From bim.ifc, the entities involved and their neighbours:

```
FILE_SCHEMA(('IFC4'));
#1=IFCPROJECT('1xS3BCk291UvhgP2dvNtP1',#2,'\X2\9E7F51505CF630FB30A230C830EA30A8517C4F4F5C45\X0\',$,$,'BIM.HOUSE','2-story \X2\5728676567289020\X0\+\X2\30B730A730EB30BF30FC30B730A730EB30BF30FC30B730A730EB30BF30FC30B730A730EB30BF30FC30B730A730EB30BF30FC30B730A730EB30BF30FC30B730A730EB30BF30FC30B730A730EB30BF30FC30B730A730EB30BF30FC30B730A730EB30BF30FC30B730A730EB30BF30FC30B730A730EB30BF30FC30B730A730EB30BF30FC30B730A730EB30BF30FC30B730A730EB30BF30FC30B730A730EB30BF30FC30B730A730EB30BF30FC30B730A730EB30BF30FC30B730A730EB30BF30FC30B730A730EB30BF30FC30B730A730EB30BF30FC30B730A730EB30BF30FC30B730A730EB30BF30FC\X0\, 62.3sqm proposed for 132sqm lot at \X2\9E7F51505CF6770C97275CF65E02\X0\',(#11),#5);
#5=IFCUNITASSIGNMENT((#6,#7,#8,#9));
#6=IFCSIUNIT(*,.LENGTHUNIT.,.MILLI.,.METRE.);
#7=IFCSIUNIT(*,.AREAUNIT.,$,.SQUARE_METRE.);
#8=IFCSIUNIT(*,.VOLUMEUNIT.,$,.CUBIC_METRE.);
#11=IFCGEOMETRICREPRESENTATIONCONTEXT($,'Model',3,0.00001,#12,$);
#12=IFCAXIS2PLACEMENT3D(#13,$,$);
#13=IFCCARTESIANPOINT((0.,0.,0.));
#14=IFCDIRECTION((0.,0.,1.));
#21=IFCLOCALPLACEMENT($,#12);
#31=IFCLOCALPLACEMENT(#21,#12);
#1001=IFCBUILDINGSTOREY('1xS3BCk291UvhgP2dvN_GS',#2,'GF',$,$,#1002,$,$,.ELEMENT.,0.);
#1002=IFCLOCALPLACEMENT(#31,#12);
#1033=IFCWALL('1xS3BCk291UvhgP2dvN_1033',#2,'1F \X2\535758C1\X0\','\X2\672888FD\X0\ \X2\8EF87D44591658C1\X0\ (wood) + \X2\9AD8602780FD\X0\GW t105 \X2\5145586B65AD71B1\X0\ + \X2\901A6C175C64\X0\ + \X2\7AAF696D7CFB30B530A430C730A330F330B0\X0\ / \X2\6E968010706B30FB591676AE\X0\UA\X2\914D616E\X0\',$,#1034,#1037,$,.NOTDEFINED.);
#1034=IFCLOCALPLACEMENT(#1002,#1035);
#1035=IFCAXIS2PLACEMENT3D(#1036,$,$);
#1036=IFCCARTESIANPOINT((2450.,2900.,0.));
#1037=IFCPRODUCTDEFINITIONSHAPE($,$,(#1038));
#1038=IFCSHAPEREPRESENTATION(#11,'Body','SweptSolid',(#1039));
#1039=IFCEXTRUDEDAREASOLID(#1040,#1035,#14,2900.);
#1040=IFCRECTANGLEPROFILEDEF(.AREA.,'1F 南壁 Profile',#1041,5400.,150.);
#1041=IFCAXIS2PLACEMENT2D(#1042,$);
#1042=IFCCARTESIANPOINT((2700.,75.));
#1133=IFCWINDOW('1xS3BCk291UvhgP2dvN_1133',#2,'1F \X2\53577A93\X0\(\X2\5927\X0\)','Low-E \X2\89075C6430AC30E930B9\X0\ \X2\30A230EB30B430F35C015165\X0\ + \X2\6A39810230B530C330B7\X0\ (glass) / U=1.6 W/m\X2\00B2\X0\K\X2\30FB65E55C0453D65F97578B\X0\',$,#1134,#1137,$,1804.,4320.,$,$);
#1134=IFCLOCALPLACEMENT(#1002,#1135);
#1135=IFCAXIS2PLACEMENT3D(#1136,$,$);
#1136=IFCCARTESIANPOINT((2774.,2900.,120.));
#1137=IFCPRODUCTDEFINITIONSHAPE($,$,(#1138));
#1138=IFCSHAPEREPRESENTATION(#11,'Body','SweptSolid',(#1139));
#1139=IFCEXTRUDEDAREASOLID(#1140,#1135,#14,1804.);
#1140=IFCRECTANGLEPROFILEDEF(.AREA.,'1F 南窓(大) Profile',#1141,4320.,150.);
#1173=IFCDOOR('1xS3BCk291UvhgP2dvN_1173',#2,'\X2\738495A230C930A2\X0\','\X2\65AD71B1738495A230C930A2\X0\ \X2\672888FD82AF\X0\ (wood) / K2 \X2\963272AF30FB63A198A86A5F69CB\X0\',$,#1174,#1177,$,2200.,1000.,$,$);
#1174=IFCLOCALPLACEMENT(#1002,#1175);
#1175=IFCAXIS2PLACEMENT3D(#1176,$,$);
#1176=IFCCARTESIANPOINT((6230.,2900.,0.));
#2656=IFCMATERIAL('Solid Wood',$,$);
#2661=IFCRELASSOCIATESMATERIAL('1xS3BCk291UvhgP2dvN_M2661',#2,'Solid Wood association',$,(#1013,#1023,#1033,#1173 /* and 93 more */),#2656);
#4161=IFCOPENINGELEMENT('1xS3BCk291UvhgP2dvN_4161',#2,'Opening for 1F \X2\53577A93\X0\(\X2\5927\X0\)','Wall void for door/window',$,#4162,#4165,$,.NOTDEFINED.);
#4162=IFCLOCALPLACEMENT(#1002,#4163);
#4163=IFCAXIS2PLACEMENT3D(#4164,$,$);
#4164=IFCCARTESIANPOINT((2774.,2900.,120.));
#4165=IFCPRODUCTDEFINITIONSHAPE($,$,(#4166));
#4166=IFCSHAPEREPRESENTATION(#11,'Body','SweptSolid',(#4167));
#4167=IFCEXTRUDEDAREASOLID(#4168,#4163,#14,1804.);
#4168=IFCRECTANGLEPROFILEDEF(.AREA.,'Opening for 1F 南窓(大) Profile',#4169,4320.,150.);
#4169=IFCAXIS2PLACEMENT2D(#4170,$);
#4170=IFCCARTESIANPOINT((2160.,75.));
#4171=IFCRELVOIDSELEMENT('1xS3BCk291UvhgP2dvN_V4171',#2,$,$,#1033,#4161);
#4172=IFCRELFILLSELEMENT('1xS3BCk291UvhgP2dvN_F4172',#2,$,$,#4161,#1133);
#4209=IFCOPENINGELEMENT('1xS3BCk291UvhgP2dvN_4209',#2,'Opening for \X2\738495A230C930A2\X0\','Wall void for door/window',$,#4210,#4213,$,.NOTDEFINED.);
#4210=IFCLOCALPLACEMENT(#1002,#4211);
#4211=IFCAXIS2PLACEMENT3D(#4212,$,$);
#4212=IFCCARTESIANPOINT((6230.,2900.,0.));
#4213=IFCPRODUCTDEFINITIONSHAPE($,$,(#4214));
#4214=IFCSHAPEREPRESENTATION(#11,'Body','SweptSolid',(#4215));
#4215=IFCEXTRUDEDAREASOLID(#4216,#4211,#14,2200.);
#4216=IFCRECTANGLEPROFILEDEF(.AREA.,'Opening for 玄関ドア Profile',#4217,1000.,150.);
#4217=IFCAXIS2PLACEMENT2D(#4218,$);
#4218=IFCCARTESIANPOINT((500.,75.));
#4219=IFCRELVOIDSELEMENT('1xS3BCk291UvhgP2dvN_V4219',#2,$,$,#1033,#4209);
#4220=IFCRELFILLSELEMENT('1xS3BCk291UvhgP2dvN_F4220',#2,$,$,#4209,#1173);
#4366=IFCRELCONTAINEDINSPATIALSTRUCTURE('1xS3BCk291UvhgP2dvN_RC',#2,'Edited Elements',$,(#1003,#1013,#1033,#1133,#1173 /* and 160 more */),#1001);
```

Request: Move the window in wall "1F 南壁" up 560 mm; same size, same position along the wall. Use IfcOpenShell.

```python
import numpy as np
import ifcopenshell
import ifcopenshell.api.geometry
import ifcopenshell.util.placement
import ifcopenshell.util.unit

model = ifcopenshell.open("bim.ifc")
unit_scale = ifcopenshell.util.unit.calculate_unit_scale(model)

window = model.by_guid("1xS3BCk291UvhgP2dvN_1133")
opening = window.FillsVoids[0].RelatingOpeningElement
dz = 560.0

shift = np.array([0.0, 0.0, dz])
# The window is not placed relative to its opening, so move both.
for product in (opening, window):
    matrix = ifcopenshell.util.placement.get_local_placement(product.ObjectPlacement)
    matrix[:3, 3] += shift
    ifcopenshell.api.geometry.edit_object_placement(model, product=product, matrix=matrix, is_si=False)

print(f"moved by {dz * unit_scale:+.3f} m")

model.write("bim_rev.ifc")
```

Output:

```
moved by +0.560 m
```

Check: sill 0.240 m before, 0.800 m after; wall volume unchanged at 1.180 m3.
